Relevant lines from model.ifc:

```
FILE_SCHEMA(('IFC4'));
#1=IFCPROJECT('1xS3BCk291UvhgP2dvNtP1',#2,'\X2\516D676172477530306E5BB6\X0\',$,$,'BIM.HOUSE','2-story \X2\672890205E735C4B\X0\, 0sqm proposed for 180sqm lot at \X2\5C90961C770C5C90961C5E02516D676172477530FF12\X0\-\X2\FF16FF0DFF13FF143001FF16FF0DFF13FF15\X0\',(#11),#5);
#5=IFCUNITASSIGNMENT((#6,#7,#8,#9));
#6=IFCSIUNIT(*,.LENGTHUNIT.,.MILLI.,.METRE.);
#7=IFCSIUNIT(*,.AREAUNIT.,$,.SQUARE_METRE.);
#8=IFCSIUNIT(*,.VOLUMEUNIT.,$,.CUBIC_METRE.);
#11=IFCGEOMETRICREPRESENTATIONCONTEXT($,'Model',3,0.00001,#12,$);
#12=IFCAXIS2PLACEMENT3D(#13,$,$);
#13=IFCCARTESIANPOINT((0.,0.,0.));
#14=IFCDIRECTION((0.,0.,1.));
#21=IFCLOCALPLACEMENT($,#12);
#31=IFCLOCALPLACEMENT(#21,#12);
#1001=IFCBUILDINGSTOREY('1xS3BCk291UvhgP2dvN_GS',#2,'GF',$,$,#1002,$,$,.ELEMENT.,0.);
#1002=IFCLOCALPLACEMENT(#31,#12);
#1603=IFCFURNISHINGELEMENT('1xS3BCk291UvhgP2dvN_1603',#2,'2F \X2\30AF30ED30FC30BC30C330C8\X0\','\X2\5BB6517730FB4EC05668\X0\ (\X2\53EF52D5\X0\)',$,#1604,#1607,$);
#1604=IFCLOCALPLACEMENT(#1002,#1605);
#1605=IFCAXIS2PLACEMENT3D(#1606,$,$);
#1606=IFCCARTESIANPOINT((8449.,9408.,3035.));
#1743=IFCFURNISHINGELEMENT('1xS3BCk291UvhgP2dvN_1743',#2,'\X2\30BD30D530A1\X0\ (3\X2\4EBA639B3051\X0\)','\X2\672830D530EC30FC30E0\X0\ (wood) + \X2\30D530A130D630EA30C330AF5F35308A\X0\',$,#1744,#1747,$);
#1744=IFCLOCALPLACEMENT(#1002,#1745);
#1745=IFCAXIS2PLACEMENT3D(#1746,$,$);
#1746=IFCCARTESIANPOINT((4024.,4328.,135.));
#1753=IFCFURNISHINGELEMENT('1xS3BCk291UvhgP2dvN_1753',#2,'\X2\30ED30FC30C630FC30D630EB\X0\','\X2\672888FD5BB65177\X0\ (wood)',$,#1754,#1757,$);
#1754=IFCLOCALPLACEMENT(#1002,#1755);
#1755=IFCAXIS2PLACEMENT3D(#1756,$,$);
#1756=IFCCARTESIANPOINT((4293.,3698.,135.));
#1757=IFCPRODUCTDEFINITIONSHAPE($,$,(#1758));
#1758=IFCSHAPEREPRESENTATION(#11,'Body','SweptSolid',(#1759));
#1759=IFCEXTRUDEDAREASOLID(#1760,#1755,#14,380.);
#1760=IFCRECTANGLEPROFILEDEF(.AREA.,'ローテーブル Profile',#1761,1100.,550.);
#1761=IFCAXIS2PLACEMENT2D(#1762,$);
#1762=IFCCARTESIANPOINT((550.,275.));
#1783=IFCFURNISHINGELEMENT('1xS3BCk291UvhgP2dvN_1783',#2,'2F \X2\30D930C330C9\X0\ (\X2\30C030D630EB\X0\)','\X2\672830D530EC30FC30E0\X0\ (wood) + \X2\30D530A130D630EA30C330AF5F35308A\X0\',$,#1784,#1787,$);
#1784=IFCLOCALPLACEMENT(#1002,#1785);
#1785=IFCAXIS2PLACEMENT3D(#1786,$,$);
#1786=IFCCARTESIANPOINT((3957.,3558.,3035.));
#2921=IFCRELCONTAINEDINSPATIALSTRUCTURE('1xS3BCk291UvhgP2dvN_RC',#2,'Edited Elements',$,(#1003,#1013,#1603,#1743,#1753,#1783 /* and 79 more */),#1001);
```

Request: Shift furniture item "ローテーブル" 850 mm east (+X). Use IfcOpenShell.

```python
import ifcopenshell
import ifcopenshell.api.geometry
import ifcopenshell.util.placement
import ifcopenshell.util.unit

model = ifcopenshell.open("model.ifc")
unit_scale = ifcopenshell.util.unit.calculate_unit_scale(model)

item = model.by_id(1753)
matrix = ifcopenshell.util.placement.get_local_placement(item.ObjectPlacement)
matrix[0, 3] += 0.85 / unit_scale
ifcopenshell.api.geometry.edit_object_placement(model, product=item, matrix=matrix, is_si=False)

print(ifcopenshell.util.placement.get_local_placement(item.ObjectPlacement).round(3) + 0.0)

model.write("model_edited.ifc")
```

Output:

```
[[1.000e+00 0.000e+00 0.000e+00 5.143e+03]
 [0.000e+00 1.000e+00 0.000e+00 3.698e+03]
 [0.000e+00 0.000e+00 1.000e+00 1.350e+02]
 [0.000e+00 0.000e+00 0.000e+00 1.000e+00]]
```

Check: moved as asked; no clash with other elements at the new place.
